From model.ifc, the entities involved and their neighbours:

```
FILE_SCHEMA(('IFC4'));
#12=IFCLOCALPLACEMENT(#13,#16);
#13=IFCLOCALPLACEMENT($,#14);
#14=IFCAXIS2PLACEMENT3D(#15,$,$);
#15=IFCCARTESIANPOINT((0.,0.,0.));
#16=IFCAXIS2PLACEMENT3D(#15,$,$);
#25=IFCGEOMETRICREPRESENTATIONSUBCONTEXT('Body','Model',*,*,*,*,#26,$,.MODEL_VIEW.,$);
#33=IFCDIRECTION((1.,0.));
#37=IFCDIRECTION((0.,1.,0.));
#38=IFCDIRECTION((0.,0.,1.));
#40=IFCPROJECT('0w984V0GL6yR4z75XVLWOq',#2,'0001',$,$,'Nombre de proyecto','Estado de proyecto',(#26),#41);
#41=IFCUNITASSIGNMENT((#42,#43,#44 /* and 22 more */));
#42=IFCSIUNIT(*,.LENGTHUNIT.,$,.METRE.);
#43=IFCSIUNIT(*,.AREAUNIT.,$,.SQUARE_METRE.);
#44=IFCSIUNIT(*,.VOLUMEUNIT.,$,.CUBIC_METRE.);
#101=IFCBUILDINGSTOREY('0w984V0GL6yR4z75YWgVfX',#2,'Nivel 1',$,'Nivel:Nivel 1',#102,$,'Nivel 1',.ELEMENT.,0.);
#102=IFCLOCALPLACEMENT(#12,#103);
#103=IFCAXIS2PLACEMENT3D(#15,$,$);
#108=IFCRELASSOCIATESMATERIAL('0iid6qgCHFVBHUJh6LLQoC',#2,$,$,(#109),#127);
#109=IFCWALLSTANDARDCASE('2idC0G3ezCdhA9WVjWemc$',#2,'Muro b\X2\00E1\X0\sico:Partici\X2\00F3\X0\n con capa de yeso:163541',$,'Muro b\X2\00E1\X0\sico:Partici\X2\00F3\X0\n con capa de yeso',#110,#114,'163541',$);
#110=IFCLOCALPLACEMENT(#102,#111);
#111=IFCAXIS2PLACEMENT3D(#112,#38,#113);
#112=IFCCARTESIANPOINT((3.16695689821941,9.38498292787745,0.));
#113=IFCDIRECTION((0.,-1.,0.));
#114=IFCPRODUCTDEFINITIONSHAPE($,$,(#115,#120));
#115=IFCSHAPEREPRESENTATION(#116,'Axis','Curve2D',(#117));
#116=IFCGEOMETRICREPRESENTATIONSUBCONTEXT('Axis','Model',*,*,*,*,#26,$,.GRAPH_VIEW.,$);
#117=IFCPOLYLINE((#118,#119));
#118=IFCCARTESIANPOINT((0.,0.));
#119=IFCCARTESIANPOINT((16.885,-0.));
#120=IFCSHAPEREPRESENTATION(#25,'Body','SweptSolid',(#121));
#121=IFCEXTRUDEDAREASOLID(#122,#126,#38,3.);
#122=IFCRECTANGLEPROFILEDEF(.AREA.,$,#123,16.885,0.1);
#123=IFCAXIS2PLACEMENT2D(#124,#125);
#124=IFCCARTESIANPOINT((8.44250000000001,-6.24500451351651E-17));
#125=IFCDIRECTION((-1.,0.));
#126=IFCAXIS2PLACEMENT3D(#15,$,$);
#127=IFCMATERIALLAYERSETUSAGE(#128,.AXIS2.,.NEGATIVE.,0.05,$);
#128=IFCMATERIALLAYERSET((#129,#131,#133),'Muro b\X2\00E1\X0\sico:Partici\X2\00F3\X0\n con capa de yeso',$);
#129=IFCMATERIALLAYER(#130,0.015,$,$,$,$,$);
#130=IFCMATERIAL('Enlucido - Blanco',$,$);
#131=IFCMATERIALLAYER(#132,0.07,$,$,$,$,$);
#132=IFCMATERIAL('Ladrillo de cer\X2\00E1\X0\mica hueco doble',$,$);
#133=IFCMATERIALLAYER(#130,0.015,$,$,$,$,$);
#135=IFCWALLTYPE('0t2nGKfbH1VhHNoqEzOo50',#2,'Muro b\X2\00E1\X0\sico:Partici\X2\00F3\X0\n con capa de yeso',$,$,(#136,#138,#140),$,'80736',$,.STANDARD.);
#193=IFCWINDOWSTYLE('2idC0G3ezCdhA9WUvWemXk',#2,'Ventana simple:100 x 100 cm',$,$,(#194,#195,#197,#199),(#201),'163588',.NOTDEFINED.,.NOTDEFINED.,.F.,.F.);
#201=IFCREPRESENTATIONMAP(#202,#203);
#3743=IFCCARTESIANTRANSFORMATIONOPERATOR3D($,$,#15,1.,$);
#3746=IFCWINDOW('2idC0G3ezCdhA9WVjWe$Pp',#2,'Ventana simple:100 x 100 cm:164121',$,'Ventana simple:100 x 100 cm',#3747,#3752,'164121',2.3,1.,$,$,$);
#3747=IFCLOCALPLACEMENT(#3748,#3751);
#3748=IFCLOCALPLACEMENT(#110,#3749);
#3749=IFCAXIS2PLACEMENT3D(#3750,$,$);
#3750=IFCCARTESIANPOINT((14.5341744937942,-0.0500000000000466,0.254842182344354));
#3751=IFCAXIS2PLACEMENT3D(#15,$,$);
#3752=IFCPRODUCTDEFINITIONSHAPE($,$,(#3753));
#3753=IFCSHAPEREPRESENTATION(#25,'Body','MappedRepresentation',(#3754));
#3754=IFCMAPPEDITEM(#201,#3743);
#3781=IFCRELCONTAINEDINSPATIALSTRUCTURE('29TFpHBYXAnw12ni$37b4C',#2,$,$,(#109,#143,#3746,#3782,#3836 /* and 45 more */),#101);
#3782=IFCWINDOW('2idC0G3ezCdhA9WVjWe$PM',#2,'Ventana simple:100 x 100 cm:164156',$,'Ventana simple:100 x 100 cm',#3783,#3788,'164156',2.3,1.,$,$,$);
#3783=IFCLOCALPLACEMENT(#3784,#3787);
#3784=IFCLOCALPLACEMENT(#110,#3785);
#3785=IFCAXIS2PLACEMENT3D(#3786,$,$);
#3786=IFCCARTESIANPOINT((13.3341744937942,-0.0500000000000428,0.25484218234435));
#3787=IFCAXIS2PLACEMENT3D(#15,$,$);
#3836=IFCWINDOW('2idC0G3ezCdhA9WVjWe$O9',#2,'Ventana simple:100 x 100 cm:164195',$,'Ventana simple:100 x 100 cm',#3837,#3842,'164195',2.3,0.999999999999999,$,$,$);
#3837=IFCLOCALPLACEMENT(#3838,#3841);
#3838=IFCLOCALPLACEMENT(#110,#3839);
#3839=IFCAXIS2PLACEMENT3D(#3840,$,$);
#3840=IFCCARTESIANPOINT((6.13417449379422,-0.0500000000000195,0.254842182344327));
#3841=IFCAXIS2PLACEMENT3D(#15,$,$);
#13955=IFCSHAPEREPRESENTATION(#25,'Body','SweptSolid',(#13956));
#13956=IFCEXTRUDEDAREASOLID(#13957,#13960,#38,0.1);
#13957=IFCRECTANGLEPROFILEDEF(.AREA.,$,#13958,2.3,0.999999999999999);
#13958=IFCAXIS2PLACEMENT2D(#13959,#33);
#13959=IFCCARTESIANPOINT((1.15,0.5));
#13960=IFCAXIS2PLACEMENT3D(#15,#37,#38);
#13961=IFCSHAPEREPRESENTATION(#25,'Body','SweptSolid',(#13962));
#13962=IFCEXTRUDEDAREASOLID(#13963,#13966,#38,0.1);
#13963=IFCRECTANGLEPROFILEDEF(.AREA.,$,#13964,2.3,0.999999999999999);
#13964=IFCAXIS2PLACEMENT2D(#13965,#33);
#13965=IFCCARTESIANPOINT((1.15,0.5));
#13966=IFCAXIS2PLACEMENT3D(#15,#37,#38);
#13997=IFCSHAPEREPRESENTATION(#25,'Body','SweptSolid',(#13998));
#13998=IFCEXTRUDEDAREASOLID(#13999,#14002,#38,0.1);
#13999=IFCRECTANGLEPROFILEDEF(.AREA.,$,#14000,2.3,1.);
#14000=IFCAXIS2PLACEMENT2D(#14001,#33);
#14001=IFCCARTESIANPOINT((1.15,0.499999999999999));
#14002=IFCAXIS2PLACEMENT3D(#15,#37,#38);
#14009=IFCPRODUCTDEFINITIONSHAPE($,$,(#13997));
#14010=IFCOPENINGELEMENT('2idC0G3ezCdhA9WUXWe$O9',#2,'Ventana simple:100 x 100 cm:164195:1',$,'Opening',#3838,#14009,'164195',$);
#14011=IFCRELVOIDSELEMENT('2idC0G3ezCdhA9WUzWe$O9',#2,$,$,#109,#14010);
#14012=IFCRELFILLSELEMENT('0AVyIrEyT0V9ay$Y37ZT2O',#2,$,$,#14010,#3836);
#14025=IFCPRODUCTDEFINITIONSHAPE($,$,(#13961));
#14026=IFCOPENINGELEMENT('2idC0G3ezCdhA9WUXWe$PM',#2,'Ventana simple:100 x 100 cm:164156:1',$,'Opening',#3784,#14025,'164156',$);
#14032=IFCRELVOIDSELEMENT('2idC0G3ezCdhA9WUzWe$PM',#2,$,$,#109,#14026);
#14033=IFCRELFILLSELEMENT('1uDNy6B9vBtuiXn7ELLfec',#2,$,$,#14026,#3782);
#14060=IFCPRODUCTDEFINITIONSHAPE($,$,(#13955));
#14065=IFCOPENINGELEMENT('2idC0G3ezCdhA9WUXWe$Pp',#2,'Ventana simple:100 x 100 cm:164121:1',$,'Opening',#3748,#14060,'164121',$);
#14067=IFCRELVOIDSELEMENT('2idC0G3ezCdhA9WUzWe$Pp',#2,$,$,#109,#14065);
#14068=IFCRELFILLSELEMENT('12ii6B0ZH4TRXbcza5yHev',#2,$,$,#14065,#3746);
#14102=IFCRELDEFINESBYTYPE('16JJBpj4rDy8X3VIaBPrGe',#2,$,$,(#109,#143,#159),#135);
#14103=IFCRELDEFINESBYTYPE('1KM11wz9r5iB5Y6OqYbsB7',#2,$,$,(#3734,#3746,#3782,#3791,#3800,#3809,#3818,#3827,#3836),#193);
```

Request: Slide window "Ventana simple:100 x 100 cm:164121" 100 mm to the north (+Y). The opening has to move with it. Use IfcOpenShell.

```python
import ifcopenshell
import ifcopenshell.api.geometry
import ifcopenshell.util.placement

model = ifcopenshell.open("model.ifc")

window = model.by_guid("2idC0G3ezCdhA9WVjWe$Pp")
opening = window.FillsVoids[0].RelatingOpeningElement
wall = opening.VoidsElements[0].RelatingBuildingElement

wall_matrix = ifcopenshell.util.placement.get_local_placement(wall.ObjectPlacement)
shift = wall_matrix[:3, 0] * -0.1
before = ifcopenshell.util.placement.get_local_placement(window.ObjectPlacement)[:3, 3].copy()

# The window is placed relative to its opening, so it follows when the opening moves.
matrix = ifcopenshell.util.placement.get_local_placement(opening.ObjectPlacement)
matrix[:3, 3] += shift
ifcopenshell.api.geometry.edit_object_placement(
    model, product=opening, matrix=matrix, is_si=False, should_transform_children=True
)

after = ifcopenshell.util.placement.get_local_placement(window.ObjectPlacement)[:3, 3]
print("window moved by", (after - before).round(3) + 0.0)

model.write("model-out.ifc")
```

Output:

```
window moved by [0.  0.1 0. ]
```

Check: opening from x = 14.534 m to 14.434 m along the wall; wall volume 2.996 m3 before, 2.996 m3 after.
